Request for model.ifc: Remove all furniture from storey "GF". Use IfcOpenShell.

First a look at what the model holds.

```python
import ifcopenshell
import ifcopenshell.util.element

model = ifcopenshell.open("model.ifc")
print(model.schema)
storey = next(s for s in model.by_type("IfcBuildingStorey") if s.Name == "GF")
furniture = [e for e in ifcopenshell.util.element.get_decomposition(storey) if e.is_a("IfcFurnishingElement")]
seen = {}
for e in furniture:
    element_type = ifcopenshell.util.element.get_type(e)
    name = element_type.Name if element_type not in (None, e) else None
    seen[name] = seen.get(name, 0) + 1
for name, count in sorted(seen.items(), key=str):
    print(count, "x", name)
```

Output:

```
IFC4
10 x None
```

```python
import ifcopenshell
import ifcopenshell.api.root
import ifcopenshell.util.element

model = ifcopenshell.open("model.ifc")

storey = next(s for s in model.by_type("IfcBuildingStorey") if s.Name == "GF")
furniture = [e for e in ifcopenshell.util.element.get_decomposition(storey) if e.is_a("IfcFurnishingElement")]

for e in furniture:
    ifcopenshell.api.root.remove_product(model, product=e)
print(len(furniture), "removed")

model.write("model-out.ifc")
```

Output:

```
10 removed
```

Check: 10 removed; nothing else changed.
